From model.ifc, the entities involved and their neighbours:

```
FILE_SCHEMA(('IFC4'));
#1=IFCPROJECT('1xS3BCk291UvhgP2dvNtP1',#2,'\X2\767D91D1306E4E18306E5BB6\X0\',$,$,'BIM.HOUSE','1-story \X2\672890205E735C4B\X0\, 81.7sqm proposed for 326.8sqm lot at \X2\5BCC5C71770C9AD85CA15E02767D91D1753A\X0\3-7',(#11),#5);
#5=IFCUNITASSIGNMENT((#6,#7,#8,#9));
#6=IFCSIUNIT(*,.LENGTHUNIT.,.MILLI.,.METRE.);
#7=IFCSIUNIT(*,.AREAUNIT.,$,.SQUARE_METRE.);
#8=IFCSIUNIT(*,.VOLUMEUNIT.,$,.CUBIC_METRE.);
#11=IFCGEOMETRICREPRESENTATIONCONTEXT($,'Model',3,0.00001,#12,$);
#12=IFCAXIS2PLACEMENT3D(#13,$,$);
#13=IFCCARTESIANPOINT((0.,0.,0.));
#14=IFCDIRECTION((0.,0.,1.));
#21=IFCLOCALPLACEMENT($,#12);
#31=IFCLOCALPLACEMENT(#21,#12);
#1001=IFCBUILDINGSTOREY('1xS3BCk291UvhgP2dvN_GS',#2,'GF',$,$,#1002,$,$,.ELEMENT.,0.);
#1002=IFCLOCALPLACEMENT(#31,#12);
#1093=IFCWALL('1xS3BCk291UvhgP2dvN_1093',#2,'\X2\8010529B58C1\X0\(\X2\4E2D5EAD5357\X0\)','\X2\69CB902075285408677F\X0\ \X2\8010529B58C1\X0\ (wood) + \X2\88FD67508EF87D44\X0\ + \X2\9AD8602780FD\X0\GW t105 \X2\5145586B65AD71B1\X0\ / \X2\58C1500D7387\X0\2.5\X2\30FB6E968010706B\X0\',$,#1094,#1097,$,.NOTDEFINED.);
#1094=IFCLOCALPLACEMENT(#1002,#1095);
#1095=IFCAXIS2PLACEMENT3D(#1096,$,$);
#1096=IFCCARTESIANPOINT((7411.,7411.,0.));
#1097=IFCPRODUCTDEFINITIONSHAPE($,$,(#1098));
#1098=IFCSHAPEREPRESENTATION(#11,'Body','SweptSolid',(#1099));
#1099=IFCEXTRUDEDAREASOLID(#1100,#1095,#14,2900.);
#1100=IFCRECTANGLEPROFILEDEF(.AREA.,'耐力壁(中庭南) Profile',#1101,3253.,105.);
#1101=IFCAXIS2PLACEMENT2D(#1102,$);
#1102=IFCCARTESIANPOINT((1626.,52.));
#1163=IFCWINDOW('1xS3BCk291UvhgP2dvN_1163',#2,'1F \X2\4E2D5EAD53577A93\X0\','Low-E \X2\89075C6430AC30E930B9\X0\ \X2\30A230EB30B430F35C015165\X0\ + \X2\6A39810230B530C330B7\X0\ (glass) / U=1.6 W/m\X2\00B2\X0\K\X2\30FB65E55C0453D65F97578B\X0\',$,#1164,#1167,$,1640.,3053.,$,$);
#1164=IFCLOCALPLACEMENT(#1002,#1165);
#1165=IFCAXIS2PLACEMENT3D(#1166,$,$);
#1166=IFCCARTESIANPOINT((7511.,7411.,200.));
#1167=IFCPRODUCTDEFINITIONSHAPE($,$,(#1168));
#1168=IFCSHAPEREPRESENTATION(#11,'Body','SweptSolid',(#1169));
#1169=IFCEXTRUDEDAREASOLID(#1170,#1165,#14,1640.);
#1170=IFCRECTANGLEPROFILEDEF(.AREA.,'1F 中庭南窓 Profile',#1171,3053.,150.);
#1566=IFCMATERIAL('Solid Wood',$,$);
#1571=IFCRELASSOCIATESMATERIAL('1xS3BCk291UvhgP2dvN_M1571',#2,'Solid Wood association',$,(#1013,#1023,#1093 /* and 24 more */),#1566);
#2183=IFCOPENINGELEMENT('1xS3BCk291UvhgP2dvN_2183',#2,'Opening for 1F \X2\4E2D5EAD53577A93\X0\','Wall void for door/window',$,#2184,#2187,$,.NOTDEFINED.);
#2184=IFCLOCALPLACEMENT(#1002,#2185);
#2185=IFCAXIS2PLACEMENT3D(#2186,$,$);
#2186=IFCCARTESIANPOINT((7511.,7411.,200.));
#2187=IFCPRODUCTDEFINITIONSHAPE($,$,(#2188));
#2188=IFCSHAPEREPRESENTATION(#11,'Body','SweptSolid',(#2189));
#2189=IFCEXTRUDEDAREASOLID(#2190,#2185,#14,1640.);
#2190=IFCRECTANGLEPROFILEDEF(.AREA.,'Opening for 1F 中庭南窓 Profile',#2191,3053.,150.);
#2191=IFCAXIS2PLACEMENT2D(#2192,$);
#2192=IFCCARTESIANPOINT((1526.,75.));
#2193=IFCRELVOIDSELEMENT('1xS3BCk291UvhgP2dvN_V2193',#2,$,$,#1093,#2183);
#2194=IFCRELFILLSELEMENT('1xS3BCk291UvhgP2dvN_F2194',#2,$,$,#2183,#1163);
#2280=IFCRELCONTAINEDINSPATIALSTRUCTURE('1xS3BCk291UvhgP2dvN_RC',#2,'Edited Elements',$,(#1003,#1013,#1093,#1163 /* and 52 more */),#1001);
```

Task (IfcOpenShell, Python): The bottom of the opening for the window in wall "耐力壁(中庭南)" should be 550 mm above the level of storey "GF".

```python
import numpy as np
import ifcopenshell
import ifcopenshell.api.geometry
import ifcopenshell.geom
import ifcopenshell.util.element
import ifcopenshell.util.placement
import ifcopenshell.util.shape
import ifcopenshell.util.unit

model = ifcopenshell.open("model.ifc")
unit_scale = ifcopenshell.util.unit.calculate_unit_scale(model)

window = model.by_id(1163)
opening = window.FillsVoids[0].RelatingOpeningElement
storey = ifcopenshell.util.element.get_container(window, ifc_class="IfcBuildingStorey")
level = ifcopenshell.util.placement.get_local_placement(storey.ObjectPlacement)[2, 3]

# The opening's origin need not be at the sill, so measure its lowest point.
shape = ifcopenshell.geom.create_shape(ifcopenshell.geom.settings(), opening)
bottom = ifcopenshell.util.shape.get_shape_bottom_elevation(shape, shape.geometry) / unit_scale
dz = level + 550.0 - bottom

shift = np.array([0.0, 0.0, dz])
# The window is not placed relative to its opening, so move both.
for product in (opening, window):
    matrix = ifcopenshell.util.placement.get_local_placement(product.ObjectPlacement)
    matrix[:3, 3] += shift
    ifcopenshell.api.geometry.edit_object_placement(model, product=product, matrix=matrix, is_si=False)

print(f"moved by {dz * unit_scale:+.3f} m")

model.write("model_edited.ifc")
```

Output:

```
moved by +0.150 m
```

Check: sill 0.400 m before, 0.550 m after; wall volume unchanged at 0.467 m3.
